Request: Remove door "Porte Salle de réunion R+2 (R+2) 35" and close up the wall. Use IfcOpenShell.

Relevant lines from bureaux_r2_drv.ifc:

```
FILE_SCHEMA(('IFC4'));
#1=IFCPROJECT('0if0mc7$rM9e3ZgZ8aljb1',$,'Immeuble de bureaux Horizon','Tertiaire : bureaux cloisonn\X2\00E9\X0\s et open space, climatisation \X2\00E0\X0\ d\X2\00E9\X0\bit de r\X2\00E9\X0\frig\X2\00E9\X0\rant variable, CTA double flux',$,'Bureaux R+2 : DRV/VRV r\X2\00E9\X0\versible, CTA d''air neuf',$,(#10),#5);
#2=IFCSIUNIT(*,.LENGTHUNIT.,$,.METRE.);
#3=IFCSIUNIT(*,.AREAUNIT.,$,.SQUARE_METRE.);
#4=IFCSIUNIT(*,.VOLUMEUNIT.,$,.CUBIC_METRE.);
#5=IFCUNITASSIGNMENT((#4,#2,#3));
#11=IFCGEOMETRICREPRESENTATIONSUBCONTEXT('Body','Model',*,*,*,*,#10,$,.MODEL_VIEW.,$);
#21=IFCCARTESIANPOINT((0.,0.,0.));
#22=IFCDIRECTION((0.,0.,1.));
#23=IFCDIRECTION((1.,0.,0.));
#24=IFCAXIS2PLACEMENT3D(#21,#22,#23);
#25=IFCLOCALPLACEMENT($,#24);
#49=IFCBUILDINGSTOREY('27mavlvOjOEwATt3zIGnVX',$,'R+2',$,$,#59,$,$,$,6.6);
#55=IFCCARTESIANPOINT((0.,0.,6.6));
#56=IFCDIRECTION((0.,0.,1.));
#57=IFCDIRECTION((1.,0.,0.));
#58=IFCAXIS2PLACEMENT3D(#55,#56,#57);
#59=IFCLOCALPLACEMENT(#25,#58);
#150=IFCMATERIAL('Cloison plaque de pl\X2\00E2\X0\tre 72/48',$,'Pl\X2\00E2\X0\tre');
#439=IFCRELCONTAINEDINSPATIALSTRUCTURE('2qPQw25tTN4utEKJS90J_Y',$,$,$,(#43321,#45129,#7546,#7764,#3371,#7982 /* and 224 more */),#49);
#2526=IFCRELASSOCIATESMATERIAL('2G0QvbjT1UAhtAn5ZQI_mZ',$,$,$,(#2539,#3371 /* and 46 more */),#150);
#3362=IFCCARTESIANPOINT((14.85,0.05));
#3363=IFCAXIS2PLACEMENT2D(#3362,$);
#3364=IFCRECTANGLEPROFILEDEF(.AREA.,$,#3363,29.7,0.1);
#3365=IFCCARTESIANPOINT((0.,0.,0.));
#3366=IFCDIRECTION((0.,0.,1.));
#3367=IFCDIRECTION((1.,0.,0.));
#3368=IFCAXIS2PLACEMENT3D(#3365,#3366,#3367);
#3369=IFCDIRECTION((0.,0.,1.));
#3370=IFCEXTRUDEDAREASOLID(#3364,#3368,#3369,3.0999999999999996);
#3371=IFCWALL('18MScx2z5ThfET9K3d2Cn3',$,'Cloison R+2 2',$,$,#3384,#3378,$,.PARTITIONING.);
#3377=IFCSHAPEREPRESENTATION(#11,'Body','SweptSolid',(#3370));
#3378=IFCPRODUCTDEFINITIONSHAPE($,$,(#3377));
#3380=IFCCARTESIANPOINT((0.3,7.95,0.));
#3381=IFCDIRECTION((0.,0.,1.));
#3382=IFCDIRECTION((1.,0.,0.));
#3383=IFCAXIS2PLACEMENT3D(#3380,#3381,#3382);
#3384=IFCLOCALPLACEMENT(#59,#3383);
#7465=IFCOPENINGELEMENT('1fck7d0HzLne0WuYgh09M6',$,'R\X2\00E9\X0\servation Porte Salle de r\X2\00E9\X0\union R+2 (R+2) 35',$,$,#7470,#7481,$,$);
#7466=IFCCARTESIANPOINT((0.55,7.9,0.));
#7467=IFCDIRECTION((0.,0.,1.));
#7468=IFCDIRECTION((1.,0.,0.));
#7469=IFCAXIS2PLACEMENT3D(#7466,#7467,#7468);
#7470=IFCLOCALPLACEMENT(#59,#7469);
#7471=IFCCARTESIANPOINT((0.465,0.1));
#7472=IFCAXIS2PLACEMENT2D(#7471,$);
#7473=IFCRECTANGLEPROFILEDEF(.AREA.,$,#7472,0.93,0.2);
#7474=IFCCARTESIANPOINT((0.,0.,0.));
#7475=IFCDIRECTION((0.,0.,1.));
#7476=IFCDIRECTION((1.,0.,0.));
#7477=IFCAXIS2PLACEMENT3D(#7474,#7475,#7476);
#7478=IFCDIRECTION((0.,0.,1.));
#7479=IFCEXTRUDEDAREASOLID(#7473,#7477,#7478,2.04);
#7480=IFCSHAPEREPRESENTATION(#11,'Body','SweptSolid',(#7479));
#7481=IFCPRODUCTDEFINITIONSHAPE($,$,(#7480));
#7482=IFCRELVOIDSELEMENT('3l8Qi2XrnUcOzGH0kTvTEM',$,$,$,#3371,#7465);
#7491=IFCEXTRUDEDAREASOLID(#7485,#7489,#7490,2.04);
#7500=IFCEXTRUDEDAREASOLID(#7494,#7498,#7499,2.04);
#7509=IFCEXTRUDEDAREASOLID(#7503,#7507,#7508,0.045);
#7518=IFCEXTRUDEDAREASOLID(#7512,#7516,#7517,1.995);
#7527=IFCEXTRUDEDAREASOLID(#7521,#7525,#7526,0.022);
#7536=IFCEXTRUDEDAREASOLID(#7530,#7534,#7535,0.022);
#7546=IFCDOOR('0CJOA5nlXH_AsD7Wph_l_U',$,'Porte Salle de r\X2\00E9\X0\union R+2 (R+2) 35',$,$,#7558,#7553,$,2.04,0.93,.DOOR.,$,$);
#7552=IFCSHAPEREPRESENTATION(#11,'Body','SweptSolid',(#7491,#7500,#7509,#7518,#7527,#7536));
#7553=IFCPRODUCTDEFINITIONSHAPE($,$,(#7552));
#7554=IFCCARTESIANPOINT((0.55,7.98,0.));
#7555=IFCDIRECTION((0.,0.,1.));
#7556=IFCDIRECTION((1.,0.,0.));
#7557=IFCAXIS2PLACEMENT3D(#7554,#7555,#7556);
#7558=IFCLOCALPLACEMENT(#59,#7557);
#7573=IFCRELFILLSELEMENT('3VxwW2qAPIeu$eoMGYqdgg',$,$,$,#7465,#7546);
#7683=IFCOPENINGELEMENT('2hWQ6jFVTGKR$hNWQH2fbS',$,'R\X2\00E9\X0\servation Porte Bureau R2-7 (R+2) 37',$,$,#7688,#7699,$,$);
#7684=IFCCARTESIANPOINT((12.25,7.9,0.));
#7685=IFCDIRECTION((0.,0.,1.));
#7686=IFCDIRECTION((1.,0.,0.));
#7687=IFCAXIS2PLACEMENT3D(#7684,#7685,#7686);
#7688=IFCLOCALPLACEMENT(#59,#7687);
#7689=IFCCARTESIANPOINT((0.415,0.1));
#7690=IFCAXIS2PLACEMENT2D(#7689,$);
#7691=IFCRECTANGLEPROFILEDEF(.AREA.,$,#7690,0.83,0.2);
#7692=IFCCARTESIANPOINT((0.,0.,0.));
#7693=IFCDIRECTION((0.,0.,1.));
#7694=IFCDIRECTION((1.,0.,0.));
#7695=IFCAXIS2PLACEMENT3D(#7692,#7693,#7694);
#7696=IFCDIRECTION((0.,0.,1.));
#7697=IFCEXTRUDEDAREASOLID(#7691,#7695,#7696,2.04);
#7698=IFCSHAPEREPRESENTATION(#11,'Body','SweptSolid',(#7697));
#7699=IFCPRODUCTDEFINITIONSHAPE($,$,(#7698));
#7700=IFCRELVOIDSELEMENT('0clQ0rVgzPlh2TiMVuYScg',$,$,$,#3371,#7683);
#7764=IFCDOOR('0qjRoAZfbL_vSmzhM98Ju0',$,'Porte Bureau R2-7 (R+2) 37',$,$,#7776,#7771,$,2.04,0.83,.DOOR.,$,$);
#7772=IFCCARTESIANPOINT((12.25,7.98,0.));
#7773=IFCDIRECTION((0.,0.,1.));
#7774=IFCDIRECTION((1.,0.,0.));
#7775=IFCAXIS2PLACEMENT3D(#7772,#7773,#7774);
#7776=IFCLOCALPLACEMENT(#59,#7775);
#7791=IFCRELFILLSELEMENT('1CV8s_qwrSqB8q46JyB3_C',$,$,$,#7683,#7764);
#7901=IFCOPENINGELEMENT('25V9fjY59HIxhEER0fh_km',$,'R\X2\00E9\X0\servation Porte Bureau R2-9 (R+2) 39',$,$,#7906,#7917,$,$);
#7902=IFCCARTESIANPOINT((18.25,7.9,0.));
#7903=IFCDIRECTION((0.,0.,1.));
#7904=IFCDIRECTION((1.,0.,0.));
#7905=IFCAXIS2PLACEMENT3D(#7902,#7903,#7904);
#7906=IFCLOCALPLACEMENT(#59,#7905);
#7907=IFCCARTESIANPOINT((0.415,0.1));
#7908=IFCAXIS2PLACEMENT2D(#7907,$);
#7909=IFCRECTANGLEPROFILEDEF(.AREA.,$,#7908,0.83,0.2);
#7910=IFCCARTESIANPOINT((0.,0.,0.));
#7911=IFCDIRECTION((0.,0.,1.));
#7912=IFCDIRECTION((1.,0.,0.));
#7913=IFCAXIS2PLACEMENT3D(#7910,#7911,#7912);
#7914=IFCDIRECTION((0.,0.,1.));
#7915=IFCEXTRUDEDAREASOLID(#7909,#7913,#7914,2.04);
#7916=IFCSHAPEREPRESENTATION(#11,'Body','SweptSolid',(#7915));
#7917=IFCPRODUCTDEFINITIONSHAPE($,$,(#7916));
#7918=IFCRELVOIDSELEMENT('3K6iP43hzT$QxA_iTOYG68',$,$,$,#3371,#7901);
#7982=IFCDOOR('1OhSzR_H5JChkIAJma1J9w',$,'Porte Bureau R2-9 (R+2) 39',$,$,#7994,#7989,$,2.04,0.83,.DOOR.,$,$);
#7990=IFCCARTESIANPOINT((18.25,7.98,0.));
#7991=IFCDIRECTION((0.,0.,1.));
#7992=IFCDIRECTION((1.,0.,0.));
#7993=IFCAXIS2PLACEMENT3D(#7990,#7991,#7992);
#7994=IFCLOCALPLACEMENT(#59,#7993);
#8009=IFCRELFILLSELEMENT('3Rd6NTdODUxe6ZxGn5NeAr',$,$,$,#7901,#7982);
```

```python
import ifcopenshell
import ifcopenshell.api.feature
import ifcopenshell.api.root
import ifcopenshell.geom
import ifcopenshell.util.shape

model = ifcopenshell.open("bureaux_r2_drv.ifc")
settings = ifcopenshell.geom.settings()


def volume(element):
    """Net volume in cubic metres, openings subtracted."""
    shape = ifcopenshell.geom.create_shape(settings, element)
    return ifcopenshell.util.shape.get_volume(shape.geometry)


door = model.by_id(7546)
opening = door.FillsVoids[0].RelatingOpeningElement
wall = opening.VoidsElements[0].RelatingBuildingElement
before = volume(wall)

ifcopenshell.api.root.remove_product(model, product=door)
ifcopenshell.api.feature.remove_feature(model, feature=opening)

after = volume(wall)

print(f"wall volume {before:.3f} -> {after:.3f} m3")

model.write("bureaux_r2_drv_v2.ifc")
```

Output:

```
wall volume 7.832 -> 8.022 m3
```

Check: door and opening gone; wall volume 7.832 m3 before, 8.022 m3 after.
